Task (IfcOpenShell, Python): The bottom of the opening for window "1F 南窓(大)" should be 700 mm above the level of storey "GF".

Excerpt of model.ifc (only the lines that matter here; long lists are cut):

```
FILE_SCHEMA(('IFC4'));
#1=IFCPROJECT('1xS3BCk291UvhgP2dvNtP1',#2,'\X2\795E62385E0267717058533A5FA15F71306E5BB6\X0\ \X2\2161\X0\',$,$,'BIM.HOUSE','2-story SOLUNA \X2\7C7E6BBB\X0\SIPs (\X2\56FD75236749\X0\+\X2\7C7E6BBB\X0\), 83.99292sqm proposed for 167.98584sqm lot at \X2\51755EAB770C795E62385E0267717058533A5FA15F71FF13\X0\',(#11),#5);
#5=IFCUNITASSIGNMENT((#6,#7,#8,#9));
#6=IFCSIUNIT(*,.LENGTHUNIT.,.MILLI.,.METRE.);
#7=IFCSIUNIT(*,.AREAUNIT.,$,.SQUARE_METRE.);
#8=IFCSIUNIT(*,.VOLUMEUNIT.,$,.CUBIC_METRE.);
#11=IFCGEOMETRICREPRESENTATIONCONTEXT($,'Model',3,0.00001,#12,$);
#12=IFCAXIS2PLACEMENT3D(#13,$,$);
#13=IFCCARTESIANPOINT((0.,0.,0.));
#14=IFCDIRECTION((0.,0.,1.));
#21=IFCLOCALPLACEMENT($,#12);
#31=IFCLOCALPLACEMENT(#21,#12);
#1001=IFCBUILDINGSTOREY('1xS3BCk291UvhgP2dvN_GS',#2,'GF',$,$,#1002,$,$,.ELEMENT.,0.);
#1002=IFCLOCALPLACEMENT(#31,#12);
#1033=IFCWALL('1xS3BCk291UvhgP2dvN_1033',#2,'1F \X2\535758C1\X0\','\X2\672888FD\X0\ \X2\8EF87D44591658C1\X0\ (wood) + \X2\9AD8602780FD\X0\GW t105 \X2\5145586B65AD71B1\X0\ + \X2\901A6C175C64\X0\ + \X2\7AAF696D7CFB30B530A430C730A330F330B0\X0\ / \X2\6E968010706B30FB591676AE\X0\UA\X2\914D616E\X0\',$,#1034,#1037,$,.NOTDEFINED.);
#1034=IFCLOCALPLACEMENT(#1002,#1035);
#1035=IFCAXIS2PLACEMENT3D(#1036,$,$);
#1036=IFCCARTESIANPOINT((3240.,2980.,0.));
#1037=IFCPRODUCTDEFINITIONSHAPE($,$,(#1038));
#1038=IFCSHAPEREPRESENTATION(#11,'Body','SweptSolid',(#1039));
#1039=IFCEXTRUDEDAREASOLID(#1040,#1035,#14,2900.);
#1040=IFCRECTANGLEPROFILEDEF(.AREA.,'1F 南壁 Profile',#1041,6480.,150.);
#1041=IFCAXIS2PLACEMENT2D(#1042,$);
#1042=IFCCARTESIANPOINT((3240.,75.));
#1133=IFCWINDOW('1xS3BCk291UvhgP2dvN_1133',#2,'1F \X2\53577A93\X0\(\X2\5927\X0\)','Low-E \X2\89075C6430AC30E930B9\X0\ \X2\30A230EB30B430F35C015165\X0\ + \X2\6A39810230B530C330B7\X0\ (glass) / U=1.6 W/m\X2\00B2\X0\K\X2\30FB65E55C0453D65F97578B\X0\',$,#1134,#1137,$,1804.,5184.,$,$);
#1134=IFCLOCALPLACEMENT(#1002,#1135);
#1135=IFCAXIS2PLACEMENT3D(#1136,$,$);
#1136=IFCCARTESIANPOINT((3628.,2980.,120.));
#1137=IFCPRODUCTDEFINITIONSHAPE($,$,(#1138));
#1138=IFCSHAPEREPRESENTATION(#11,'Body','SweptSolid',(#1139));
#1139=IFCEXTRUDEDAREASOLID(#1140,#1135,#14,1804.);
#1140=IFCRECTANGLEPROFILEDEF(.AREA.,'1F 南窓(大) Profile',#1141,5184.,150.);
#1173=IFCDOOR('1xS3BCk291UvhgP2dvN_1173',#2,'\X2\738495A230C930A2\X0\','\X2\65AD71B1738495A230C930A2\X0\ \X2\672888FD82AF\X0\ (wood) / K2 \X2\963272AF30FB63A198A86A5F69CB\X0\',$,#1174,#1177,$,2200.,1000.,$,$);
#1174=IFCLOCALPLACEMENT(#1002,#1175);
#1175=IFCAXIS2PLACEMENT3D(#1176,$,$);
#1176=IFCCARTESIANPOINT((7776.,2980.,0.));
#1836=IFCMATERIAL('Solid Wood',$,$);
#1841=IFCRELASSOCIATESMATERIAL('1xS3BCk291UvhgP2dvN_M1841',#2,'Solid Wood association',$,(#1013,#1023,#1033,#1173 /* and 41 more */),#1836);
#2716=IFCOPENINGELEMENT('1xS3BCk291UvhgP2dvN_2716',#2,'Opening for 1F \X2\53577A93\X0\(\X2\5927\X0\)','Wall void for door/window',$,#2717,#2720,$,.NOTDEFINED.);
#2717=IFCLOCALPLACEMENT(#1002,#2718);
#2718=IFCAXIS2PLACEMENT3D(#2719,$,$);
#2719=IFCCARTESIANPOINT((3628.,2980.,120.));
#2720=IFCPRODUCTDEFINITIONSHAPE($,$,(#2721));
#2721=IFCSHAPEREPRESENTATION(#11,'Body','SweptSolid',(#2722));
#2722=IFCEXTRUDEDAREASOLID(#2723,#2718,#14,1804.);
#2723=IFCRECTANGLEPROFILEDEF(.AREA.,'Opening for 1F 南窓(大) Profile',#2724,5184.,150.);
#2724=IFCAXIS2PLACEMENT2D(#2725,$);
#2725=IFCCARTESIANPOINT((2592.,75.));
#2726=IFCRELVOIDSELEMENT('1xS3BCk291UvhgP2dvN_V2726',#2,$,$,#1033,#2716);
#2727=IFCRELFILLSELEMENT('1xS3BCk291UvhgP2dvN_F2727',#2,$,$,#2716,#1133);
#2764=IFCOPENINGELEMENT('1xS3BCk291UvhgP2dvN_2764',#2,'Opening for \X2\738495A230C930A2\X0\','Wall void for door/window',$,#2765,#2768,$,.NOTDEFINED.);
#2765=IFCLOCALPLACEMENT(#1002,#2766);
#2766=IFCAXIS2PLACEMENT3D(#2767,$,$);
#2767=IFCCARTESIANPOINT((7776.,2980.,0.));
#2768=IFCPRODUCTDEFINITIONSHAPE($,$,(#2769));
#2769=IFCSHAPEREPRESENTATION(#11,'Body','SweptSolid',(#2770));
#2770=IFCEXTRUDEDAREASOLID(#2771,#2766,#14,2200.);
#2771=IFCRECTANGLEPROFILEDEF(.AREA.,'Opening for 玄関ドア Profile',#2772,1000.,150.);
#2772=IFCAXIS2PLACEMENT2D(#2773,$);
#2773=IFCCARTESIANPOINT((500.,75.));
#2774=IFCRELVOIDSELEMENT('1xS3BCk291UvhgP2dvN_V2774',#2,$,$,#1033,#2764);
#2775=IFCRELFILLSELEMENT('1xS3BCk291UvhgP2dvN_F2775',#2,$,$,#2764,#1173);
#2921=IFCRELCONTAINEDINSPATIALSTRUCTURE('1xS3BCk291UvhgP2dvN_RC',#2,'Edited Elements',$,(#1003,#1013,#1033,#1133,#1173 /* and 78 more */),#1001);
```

```python
import numpy as np
import ifcopenshell
import ifcopenshell.api.geometry
import ifcopenshell.geom
import ifcopenshell.util.element
import ifcopenshell.util.placement
import ifcopenshell.util.shape
import ifcopenshell.util.unit

model = ifcopenshell.open("model.ifc")
unit_scale = ifcopenshell.util.unit.calculate_unit_scale(model)

window = model.by_guid("1xS3BCk291UvhgP2dvN_1133")
opening = window.FillsVoids[0].RelatingOpeningElement
storey = ifcopenshell.util.element.get_container(window, ifc_class="IfcBuildingStorey")
level = ifcopenshell.util.placement.get_local_placement(storey.ObjectPlacement)[2, 3]

# The opening's origin need not be at the sill, so measure its lowest point.
shape = ifcopenshell.geom.create_shape(ifcopenshell.geom.settings(), opening)
bottom = ifcopenshell.util.shape.get_shape_bottom_elevation(shape, shape.geometry) / unit_scale
dz = level + 700.0 - bottom

shift = np.array([0.0, 0.0, dz])
# The window is not placed relative to its opening, so move both.
for product in (opening, window):
    matrix = ifcopenshell.util.placement.get_local_placement(product.ObjectPlacement)
    matrix[:3, 3] += shift
    ifcopenshell.api.geometry.edit_object_placement(model, product=product, matrix=matrix, is_si=False)

print(f"moved by {dz * unit_scale:+.3f} m")

model.write("model_edited.ifc")
```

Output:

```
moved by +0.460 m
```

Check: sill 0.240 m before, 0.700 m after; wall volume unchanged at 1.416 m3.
